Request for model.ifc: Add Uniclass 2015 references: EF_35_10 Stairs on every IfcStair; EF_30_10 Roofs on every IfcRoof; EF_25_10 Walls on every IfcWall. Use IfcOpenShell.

First a look at what the model holds.

```python
import ifcopenshell

model = ifcopenshell.open("model.ifc")
print(model.schema)
print("classifications:", [c.Name for c in model.by_type("IfcClassification")])
for ifc_class in ("IfcDoor", "IfcRoof", "IfcStair", "IfcWall", "IfcWindow"):
    print(ifc_class, len(model.by_type(ifc_class)))
```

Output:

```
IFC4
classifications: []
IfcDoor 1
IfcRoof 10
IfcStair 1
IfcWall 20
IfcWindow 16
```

```python
import ifcopenshell
import ifcopenshell.api.classification

model = ifcopenshell.open("model.ifc")

system = ifcopenshell.api.classification.add_classification(model, classification="Uniclass 2015")

codes = {
    "IfcStair": ("EF_35_10", "Stairs"),
    "IfcRoof": ("EF_30_10", "Roofs"),
    "IfcWall": ("EF_25_10", "Walls"),
}
for ifc_class, (code, name) in codes.items():
    products = model.by_type(ifc_class)
    ifcopenshell.api.classification.add_reference(
        model, products=products, classification=system, identification=code, name=name
    )
    print(code, len(products))

model.write("model_v2.ifc")
```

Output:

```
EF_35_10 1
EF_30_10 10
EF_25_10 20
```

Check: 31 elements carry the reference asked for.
